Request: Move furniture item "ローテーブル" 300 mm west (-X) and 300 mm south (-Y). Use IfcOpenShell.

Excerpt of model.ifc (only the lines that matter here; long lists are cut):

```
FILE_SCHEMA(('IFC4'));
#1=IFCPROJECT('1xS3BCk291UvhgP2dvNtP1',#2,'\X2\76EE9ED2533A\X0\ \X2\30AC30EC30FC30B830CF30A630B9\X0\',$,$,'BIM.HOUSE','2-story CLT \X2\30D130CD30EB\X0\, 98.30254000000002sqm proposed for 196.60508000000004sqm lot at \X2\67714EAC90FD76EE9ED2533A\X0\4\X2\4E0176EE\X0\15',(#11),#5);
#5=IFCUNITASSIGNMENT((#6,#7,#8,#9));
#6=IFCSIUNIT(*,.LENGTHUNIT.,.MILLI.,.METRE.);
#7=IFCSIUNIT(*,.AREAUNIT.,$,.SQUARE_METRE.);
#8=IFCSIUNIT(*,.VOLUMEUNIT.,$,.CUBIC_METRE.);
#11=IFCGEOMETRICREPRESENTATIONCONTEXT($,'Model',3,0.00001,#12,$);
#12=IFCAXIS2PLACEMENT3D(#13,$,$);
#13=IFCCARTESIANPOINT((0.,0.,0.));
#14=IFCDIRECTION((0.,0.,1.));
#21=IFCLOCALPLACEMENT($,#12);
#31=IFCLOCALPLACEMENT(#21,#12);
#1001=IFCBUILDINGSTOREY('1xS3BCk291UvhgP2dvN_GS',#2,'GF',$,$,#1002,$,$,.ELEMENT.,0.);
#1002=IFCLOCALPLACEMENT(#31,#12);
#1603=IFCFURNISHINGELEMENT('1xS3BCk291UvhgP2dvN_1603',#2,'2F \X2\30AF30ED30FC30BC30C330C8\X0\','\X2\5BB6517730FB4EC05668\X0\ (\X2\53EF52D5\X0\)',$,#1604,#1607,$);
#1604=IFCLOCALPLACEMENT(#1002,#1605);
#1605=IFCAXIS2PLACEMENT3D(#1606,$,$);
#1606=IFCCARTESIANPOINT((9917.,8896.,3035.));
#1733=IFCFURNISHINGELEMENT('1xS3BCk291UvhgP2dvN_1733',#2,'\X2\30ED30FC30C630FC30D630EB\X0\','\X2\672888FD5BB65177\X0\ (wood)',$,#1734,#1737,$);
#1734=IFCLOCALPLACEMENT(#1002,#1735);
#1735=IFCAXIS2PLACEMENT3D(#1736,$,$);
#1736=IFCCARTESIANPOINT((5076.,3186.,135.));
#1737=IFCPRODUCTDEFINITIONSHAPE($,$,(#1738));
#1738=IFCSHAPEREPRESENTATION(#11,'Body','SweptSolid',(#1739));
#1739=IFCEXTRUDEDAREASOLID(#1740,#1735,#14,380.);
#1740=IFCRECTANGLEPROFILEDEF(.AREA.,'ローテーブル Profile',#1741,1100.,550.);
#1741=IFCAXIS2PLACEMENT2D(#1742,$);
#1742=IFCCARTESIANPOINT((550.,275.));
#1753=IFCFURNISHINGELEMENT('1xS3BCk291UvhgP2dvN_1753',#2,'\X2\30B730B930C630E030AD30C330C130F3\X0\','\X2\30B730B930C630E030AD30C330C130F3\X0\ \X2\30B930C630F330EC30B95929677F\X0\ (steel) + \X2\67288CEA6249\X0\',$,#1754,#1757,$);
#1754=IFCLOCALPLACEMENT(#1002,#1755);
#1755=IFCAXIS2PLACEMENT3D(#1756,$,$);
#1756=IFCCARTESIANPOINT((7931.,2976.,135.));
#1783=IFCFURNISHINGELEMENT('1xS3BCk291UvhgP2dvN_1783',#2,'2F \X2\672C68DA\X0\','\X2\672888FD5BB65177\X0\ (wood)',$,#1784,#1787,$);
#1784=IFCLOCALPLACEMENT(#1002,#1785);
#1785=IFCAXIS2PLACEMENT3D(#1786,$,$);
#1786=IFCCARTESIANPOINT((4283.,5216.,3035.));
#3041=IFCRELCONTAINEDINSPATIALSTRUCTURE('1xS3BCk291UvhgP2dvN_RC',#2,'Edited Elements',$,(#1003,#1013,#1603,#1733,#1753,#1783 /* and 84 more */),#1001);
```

```python
import ifcopenshell
import ifcopenshell.api.geometry
import ifcopenshell.util.placement

model = ifcopenshell.open("model.ifc")

item = model.by_guid("1xS3BCk291UvhgP2dvN_1733")
matrix = ifcopenshell.util.placement.get_local_placement(item.ObjectPlacement)
matrix[0, 3] -= 300.0
matrix[1, 3] -= 300.0
ifcopenshell.api.geometry.edit_object_placement(model, product=item, matrix=matrix, is_si=False)

print(ifcopenshell.util.placement.get_local_placement(item.ObjectPlacement).round(3) + 0.0)

model.write("model_rev.ifc")
```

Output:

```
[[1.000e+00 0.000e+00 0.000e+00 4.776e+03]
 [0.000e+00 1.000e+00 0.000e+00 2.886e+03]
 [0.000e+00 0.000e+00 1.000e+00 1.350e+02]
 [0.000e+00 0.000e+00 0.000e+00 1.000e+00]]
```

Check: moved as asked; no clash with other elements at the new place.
